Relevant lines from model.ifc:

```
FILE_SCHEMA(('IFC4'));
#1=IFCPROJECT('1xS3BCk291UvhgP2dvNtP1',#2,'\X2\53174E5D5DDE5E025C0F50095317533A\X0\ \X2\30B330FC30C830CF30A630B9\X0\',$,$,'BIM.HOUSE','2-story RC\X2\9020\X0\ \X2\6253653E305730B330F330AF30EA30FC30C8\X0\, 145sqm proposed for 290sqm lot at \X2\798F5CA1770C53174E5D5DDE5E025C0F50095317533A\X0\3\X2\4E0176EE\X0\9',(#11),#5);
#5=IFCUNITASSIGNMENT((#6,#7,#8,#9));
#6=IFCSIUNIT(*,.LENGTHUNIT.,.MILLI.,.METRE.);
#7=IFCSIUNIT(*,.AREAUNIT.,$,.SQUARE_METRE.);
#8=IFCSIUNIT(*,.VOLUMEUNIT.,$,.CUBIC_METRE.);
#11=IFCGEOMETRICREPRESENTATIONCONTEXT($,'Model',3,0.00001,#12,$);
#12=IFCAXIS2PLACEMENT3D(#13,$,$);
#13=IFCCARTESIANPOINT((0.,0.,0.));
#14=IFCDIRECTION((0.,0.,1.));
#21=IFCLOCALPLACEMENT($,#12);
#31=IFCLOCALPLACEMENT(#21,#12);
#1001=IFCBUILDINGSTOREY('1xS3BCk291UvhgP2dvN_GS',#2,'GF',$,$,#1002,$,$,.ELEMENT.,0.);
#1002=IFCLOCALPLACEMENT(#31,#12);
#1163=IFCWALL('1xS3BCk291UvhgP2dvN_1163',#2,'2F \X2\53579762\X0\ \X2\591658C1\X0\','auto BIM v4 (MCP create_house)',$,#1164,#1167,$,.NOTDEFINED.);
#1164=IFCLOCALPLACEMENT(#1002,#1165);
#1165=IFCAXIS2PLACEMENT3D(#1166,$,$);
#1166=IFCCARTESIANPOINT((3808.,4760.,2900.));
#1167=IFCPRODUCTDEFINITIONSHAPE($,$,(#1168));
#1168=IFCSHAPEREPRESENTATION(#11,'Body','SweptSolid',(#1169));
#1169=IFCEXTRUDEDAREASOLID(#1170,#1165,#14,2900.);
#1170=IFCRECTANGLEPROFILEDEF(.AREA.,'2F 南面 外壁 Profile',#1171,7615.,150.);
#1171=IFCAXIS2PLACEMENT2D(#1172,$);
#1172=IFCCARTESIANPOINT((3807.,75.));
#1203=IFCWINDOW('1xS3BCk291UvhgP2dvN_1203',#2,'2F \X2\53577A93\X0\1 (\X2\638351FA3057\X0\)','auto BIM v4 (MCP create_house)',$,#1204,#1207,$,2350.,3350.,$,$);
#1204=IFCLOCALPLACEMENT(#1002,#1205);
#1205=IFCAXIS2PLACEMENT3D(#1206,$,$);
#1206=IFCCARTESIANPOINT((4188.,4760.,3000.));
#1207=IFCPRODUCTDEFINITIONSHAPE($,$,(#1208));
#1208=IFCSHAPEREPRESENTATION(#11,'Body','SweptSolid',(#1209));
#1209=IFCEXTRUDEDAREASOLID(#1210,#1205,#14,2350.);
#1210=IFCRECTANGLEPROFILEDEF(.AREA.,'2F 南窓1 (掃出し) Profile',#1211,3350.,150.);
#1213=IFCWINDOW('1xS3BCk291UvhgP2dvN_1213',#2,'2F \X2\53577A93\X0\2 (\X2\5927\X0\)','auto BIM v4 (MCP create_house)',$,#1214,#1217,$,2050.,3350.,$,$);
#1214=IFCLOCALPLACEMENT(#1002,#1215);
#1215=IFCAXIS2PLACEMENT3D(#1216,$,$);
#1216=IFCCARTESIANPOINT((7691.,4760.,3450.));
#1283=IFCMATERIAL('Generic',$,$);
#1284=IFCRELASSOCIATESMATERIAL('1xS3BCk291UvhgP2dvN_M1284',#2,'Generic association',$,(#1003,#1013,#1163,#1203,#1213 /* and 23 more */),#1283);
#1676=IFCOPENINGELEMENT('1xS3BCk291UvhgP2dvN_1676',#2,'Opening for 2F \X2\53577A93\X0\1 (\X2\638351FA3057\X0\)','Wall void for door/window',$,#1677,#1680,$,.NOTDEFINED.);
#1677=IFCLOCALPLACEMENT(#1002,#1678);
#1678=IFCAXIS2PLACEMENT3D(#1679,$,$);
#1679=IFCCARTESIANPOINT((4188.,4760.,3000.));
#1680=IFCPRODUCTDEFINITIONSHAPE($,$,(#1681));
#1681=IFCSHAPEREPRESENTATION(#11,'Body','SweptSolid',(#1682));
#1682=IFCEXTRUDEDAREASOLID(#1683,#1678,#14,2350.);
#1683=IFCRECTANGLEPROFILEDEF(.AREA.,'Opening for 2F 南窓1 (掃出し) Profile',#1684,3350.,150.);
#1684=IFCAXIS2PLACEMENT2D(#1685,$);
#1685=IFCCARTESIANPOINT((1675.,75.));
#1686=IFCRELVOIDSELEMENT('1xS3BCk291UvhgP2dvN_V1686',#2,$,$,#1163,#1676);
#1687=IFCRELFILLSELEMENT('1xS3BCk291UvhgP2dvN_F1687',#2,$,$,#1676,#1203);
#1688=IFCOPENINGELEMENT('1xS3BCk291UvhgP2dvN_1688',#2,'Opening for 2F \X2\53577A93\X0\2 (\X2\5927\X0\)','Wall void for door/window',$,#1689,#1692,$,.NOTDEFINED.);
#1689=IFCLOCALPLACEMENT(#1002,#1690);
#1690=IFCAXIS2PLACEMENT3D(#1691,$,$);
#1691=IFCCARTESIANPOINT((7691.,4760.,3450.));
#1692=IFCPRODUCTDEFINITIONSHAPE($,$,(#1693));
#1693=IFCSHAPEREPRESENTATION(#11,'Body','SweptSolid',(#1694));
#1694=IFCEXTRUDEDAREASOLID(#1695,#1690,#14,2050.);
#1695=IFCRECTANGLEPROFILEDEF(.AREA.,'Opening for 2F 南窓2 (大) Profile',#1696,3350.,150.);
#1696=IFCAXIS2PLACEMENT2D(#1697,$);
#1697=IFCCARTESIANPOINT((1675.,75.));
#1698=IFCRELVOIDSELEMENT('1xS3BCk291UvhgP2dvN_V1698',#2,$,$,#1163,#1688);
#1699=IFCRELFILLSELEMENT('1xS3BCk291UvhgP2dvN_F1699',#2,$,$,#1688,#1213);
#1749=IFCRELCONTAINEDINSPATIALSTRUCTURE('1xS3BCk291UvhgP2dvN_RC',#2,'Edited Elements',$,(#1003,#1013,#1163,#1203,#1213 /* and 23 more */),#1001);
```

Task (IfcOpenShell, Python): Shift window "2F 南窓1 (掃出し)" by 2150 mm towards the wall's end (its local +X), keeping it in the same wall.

```python
import ifcopenshell
import ifcopenshell.api.geometry
import ifcopenshell.util.placement

model = ifcopenshell.open("model.ifc")

window = model.by_id(1203)
opening = window.FillsVoids[0].RelatingOpeningElement
wall = opening.VoidsElements[0].RelatingBuildingElement

wall_matrix = ifcopenshell.util.placement.get_local_placement(wall.ObjectPlacement)
shift = wall_matrix[:3, 0] * 2150.0
before = ifcopenshell.util.placement.get_local_placement(window.ObjectPlacement)[:3, 3].copy()

# The window is not placed relative to its opening, so move both.
for product in (opening, window):
    matrix = ifcopenshell.util.placement.get_local_placement(product.ObjectPlacement)
    matrix[:3, 3] += shift
    ifcopenshell.api.geometry.edit_object_placement(model, product=product, matrix=matrix, is_si=False)

after = ifcopenshell.util.placement.get_local_placement(window.ObjectPlacement)[:3, 3]
print("window moved by", (after - before).round(3) + 0.0)

model.write("model_v2.ifc")
```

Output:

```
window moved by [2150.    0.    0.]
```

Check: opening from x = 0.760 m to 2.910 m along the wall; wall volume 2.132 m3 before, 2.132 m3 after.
